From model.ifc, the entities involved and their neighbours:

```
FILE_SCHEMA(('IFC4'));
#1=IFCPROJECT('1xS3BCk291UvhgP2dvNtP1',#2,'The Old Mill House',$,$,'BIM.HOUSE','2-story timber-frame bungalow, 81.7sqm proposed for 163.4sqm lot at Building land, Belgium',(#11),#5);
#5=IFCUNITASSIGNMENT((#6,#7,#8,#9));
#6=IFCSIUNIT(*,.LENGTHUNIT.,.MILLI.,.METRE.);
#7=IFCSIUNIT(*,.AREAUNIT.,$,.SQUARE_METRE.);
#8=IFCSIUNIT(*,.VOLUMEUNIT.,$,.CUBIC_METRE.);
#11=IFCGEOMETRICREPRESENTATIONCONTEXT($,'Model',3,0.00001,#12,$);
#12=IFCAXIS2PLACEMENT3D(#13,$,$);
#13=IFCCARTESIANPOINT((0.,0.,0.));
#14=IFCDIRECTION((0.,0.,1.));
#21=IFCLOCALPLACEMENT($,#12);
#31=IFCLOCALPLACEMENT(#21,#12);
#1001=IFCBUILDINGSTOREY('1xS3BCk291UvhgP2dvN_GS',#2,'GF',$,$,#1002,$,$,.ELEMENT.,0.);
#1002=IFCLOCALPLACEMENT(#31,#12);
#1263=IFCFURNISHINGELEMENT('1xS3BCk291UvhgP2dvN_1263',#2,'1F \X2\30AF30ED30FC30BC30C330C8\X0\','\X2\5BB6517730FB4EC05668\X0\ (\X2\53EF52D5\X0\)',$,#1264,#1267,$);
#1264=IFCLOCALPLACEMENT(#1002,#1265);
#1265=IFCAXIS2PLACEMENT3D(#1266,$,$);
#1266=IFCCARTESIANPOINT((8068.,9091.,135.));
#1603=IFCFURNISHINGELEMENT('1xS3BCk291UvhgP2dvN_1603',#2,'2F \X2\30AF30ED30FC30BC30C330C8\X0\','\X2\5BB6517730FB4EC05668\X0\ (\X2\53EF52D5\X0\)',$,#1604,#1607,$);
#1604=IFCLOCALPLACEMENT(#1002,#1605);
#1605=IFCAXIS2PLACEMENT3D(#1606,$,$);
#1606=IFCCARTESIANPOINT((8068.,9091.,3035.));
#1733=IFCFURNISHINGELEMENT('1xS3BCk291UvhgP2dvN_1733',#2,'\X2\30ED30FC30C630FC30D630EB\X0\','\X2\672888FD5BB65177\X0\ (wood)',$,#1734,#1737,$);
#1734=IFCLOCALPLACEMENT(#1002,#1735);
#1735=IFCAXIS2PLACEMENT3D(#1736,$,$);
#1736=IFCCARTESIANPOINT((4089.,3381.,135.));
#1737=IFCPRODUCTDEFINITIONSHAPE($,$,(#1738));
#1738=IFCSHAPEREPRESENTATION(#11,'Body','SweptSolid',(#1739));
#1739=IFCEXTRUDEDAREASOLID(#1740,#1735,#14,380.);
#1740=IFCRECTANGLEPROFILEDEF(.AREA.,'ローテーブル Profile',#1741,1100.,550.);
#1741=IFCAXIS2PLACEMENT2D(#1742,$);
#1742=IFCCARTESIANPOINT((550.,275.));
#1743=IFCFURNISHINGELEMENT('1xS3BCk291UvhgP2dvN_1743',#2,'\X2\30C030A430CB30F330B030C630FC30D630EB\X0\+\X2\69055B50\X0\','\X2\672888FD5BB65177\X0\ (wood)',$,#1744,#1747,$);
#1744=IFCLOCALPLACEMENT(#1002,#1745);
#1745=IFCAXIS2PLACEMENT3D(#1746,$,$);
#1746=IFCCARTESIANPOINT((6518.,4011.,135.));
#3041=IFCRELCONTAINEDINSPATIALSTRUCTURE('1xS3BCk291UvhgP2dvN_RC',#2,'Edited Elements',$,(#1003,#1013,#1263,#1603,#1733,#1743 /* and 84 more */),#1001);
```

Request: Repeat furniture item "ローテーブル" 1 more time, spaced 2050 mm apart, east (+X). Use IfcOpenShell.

```python
import numpy as np
import ifcopenshell
import ifcopenshell.api.geometry
import ifcopenshell.api.root
import ifcopenshell.util.element
import ifcopenshell.util.placement

model = ifcopenshell.open("model.ifc")


def reuse_history(source, copy):
    """copy_class also copies each property set's owner history, people and application; keep the originals."""
    for rel in copy.IsDefinedBy:
        if rel.is_a("IfcRelDefinesByProperties") and (history := rel.RelatingPropertyDefinition.OwnerHistory):
            rel.RelatingPropertyDefinition.OwnerHistory = source.OwnerHistory
            ifcopenshell.util.element.remove_deep2(model, history)


source = model.by_guid("1xS3BCk291UvhgP2dvN_1733")
base = ifcopenshell.util.placement.get_local_placement(source.ObjectPlacement)
step = np.array([1.0, 0.0, 0.0]) * 2050.0

for i in range(1, 2):
    copy = ifcopenshell.api.root.copy_class(model, product=source)
    copy.Representation = ifcopenshell.util.element.copy_deep(
        model, source.Representation, exclude=["IfcGeometricRepresentationContext", "IfcRepresentationMap"]
    )
    reuse_history(source, copy)
    matrix = base.copy()
    matrix[:3, 3] += i * step
    print("added at", matrix[:3, 3].round(3) + 0.0)
    ifcopenshell.api.geometry.edit_object_placement(model, product=copy, matrix=matrix, is_si=False)

model.write("model_updated.ifc")
```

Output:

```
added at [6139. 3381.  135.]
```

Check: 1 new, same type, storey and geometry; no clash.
